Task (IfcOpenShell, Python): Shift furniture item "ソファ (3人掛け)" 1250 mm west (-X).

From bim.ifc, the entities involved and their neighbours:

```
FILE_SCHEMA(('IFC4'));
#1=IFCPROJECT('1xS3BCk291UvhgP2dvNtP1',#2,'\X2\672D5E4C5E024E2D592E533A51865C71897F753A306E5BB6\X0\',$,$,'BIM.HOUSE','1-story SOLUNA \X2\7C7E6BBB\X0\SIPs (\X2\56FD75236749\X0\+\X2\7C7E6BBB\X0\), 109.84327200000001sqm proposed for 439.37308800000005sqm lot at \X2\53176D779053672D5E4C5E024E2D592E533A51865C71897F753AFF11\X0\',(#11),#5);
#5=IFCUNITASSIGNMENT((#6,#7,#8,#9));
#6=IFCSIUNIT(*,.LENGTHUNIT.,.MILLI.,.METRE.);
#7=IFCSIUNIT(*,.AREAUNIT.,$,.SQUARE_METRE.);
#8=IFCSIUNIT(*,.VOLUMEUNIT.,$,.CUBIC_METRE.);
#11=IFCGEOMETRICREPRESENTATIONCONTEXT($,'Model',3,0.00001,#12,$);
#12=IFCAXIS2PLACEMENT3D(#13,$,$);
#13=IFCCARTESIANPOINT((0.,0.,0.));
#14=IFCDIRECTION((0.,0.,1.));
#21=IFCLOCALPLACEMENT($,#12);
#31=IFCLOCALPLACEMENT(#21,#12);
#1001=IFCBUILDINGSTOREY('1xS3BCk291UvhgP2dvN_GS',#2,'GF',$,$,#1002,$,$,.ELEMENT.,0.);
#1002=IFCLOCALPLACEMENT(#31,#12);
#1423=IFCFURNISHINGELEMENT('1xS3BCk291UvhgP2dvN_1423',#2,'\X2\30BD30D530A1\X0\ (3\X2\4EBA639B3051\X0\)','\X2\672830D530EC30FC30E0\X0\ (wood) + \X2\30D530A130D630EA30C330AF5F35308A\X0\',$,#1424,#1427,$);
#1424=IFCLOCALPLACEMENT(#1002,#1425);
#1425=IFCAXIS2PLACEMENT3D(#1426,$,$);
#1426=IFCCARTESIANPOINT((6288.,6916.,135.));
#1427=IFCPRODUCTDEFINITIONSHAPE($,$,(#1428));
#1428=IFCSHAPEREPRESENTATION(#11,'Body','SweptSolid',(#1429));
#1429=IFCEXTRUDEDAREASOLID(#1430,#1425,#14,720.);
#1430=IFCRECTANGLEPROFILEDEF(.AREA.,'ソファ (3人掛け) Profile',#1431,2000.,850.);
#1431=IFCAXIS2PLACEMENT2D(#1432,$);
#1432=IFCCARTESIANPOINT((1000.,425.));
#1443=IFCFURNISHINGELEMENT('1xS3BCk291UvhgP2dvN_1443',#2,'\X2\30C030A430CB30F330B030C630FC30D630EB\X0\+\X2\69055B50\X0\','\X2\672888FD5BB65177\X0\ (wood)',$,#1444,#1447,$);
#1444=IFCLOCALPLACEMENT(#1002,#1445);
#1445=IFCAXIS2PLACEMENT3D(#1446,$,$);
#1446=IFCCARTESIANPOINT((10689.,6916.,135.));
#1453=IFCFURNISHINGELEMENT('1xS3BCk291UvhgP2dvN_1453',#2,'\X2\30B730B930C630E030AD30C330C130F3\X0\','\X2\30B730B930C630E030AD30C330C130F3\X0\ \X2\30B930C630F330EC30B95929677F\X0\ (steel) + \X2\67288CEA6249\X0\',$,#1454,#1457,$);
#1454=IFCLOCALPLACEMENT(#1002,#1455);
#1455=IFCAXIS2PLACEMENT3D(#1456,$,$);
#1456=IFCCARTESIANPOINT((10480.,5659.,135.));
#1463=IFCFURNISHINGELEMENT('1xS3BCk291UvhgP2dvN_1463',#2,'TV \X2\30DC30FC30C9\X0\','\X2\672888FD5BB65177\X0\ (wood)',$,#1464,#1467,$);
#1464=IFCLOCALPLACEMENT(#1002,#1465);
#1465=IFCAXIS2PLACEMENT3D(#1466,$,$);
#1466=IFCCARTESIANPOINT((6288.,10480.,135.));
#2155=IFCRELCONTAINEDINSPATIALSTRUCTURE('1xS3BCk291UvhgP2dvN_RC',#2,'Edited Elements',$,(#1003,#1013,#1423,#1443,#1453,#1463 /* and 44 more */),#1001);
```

```python
import ifcopenshell
import ifcopenshell.api.geometry
import ifcopenshell.util.placement

model = ifcopenshell.open("bim.ifc")

item = model.by_guid("1xS3BCk291UvhgP2dvN_1423")
matrix = ifcopenshell.util.placement.get_local_placement(item.ObjectPlacement)
matrix[0, 3] -= 1250.0
ifcopenshell.api.geometry.edit_object_placement(model, product=item, matrix=matrix, is_si=False)

print(ifcopenshell.util.placement.get_local_placement(item.ObjectPlacement).round(3) + 0.0)

model.write("bim_updated.ifc")
```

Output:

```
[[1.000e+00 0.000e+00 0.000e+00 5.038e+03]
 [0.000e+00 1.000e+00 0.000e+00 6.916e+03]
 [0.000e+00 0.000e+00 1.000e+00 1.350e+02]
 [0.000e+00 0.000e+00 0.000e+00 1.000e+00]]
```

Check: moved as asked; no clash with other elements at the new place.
